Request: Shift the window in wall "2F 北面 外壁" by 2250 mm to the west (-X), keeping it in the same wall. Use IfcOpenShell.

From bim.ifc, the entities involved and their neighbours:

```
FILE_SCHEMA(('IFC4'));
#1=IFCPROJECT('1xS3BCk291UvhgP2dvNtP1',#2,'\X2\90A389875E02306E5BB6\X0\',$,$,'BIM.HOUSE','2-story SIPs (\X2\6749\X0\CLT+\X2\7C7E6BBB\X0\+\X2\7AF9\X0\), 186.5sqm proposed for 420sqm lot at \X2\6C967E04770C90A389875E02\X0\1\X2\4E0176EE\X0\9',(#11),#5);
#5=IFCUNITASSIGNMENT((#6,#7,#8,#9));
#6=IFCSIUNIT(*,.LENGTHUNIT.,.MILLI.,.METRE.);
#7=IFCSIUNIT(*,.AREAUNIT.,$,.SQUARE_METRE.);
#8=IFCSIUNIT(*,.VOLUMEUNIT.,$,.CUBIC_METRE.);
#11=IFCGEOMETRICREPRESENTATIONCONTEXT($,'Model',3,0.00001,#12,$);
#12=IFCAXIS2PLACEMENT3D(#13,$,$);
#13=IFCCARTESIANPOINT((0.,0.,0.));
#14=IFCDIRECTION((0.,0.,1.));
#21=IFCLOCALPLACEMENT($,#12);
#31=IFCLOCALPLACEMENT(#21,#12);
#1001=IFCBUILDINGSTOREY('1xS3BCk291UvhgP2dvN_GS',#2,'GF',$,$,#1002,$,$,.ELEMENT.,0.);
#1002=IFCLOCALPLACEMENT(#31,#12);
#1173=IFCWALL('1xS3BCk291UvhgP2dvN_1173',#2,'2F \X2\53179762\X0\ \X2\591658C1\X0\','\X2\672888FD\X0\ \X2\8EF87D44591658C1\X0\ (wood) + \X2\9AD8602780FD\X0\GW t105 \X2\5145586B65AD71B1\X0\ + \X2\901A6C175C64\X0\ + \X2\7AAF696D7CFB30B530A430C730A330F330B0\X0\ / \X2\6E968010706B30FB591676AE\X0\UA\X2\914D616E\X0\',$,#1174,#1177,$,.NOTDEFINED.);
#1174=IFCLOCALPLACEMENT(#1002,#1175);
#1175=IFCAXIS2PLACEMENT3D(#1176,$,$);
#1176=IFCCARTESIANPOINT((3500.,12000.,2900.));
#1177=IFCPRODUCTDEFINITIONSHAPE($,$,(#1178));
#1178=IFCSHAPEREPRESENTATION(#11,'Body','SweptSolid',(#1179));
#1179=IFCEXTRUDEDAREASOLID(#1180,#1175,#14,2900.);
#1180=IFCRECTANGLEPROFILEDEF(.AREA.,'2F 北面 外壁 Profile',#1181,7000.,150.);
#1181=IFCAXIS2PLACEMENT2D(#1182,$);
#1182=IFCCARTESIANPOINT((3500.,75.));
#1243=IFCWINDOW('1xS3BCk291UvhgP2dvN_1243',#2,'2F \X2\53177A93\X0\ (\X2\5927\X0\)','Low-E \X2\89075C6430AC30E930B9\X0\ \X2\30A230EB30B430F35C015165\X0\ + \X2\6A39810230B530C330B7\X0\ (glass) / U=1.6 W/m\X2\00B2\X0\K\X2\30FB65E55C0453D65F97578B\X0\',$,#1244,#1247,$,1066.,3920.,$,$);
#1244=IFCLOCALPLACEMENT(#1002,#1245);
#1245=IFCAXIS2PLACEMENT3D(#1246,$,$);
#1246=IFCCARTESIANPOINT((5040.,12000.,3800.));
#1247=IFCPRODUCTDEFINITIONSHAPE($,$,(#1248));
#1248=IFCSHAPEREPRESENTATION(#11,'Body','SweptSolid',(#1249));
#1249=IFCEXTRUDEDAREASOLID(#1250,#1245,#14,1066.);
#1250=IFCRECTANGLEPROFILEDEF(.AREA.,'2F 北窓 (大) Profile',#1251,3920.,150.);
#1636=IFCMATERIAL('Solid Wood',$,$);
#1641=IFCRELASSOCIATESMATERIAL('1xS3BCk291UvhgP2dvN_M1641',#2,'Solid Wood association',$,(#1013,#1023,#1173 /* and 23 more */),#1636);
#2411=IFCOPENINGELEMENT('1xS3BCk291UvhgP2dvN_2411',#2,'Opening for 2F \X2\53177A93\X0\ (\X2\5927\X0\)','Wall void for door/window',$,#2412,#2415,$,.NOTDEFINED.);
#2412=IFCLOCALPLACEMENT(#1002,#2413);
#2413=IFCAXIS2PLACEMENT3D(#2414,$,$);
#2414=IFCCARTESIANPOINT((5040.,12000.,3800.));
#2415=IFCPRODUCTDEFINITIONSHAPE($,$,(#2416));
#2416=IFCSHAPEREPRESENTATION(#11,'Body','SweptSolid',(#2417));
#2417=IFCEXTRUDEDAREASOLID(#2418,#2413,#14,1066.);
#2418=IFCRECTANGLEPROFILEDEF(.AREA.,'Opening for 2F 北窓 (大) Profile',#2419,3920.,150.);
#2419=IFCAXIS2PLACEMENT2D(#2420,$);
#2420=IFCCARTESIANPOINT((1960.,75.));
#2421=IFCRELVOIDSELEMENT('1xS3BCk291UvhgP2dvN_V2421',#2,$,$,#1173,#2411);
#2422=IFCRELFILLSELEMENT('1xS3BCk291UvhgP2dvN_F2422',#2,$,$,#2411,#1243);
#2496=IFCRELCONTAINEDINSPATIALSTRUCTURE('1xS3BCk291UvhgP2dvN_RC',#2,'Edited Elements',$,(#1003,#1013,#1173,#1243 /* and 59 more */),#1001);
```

```python
import ifcopenshell
import ifcopenshell.api.geometry
import ifcopenshell.util.placement
import ifcopenshell.util.unit

model = ifcopenshell.open("bim.ifc")
unit_scale = ifcopenshell.util.unit.calculate_unit_scale(model)

window = model.by_id(1243)
opening = window.FillsVoids[0].RelatingOpeningElement
wall = opening.VoidsElements[0].RelatingBuildingElement

wall_matrix = ifcopenshell.util.placement.get_local_placement(wall.ObjectPlacement)
shift = wall_matrix[:3, 0] * -2.25 / unit_scale
before = ifcopenshell.util.placement.get_local_placement(window.ObjectPlacement)[:3, 3].copy()

# The window is not placed relative to its opening, so move both.
for product in (opening, window):
    matrix = ifcopenshell.util.placement.get_local_placement(product.ObjectPlacement)
    matrix[:3, 3] += shift
    ifcopenshell.api.geometry.edit_object_placement(model, product=product, matrix=matrix, is_si=False)

after = ifcopenshell.util.placement.get_local_placement(window.ObjectPlacement)[:3, 3]
print("window moved by", (after - before).round(3) + 0.0)

model.write("bim-out.ifc")
```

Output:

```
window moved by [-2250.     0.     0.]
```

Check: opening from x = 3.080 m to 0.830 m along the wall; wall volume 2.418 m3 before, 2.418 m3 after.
